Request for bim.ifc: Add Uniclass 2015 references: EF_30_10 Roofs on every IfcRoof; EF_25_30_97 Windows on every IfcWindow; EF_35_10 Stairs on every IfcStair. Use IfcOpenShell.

First a look at what the model holds.

```python
import ifcopenshell

model = ifcopenshell.open("bim.ifc")
print(model.schema)
print("classifications:", [c.Name for c in model.by_type("IfcClassification")])
for ifc_class in ("IfcDoor", "IfcRoof", "IfcStair", "IfcWall", "IfcWindow"):
    print(ifc_class, len(model.by_type(ifc_class)))
```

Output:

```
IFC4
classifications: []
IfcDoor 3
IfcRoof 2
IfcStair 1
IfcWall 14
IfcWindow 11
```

```python
import ifcopenshell
import ifcopenshell.api.classification

model = ifcopenshell.open("bim.ifc")

system = ifcopenshell.api.classification.add_classification(model, classification="Uniclass 2015")

codes = {
    "IfcRoof": ("EF_30_10", "Roofs"),
    "IfcWindow": ("EF_25_30_97", "Windows"),
    "IfcStair": ("EF_35_10", "Stairs"),
}
for ifc_class, (code, name) in codes.items():
    products = model.by_type(ifc_class)
    ifcopenshell.api.classification.add_reference(
        model, products=products, classification=system, identification=code, name=name
    )
    print(code, len(products))

model.write("bim_v2.ifc")
```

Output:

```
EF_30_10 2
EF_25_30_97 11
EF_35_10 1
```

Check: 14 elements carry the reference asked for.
